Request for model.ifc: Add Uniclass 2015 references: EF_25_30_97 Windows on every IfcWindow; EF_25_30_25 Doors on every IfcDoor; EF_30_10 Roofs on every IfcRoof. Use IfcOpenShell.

First a look at what the model holds.

```python
import ifcopenshell

model = ifcopenshell.open("model.ifc")
print(model.schema)
print("classifications:", [c.Name for c in model.by_type("IfcClassification")])
for ifc_class in ("IfcDoor", "IfcRoof", "IfcStair", "IfcWall", "IfcWindow"):
    print(ifc_class, len(model.by_type(ifc_class)))
```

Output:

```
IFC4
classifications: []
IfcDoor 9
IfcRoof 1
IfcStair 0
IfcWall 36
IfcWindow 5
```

```python
import ifcopenshell
import ifcopenshell.api.classification

model = ifcopenshell.open("model.ifc")

system = ifcopenshell.api.classification.add_classification(model, classification="Uniclass 2015")

codes = {
    "IfcWindow": ("EF_25_30_97", "Windows"),
    "IfcDoor": ("EF_25_30_25", "Doors"),
    "IfcRoof": ("EF_30_10", "Roofs"),
}
for ifc_class, (code, name) in codes.items():
    products = model.by_type(ifc_class)
    ifcopenshell.api.classification.add_reference(
        model, products=products, classification=system, identification=code, name=name
    )
    print(code, len(products))

model.write("model_rev.ifc")
```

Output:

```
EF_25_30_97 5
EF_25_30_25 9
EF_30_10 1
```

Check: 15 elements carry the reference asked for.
